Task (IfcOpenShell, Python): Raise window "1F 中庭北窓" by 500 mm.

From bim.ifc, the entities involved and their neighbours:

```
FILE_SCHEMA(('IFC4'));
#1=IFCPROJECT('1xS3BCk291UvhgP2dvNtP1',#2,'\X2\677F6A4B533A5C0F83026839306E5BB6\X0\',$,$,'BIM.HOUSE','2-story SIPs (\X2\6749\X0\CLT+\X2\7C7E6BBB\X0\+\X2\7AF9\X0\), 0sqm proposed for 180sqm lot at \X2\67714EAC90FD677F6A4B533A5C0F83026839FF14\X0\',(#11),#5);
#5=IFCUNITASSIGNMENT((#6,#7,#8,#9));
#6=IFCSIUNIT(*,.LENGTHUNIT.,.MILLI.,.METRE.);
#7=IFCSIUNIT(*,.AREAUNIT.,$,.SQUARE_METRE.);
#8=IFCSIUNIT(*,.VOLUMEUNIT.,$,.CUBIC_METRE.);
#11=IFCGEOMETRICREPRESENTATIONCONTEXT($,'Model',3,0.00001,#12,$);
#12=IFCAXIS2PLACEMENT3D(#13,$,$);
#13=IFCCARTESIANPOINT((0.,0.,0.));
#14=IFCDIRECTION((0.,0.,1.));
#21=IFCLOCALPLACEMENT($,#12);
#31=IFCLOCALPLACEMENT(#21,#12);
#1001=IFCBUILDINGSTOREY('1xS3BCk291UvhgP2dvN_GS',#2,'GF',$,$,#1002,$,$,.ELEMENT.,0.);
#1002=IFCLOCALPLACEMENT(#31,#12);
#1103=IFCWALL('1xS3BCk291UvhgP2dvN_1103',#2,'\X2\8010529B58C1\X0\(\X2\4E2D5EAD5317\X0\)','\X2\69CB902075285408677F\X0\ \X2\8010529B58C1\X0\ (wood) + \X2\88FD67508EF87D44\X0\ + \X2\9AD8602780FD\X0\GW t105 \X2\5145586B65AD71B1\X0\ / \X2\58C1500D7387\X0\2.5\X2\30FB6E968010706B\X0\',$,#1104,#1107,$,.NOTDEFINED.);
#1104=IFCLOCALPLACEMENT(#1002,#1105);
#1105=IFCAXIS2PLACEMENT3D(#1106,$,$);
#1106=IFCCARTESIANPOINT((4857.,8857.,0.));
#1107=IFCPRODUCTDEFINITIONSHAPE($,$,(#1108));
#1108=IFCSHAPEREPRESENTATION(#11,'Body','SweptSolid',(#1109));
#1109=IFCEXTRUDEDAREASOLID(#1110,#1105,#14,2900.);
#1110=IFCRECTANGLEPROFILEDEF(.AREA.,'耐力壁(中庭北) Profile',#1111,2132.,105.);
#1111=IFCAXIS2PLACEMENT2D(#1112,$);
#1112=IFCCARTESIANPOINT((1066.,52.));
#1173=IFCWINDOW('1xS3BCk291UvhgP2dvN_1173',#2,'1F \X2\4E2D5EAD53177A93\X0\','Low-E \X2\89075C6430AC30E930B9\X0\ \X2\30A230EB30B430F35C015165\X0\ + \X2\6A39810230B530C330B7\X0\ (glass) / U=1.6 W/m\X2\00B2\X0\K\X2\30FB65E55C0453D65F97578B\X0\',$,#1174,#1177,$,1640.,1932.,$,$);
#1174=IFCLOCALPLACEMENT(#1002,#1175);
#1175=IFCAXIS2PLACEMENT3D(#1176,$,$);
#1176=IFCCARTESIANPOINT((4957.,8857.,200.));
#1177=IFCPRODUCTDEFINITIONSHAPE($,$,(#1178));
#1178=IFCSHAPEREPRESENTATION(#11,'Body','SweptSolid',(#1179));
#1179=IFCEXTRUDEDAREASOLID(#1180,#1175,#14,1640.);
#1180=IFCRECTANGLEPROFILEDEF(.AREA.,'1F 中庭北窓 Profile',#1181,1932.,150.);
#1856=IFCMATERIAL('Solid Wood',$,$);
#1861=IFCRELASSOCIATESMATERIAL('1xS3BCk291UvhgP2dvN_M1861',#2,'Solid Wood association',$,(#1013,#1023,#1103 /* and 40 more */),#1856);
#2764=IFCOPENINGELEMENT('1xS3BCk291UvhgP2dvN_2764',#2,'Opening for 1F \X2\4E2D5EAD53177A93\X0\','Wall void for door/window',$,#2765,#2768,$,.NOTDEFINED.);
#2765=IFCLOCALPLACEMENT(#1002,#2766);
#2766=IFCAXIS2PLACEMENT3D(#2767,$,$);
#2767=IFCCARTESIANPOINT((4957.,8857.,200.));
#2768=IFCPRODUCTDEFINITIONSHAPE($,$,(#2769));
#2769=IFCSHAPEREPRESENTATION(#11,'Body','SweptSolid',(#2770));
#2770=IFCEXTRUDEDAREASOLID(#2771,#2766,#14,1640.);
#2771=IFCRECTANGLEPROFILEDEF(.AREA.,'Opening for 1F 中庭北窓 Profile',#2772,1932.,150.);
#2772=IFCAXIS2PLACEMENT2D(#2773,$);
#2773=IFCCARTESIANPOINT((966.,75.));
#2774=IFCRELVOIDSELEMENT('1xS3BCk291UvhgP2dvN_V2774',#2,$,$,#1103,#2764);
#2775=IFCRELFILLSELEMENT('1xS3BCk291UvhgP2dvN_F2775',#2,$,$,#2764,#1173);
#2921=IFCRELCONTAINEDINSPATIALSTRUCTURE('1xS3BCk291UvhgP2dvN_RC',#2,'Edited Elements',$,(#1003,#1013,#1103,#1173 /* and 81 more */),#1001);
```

```python
import numpy as np
import ifcopenshell
import ifcopenshell.api.geometry
import ifcopenshell.util.placement
import ifcopenshell.util.unit

model = ifcopenshell.open("bim.ifc")
unit_scale = ifcopenshell.util.unit.calculate_unit_scale(model)

window = model.by_guid("1xS3BCk291UvhgP2dvN_1173")
opening = window.FillsVoids[0].RelatingOpeningElement
dz = 0.5 / unit_scale

shift = np.array([0.0, 0.0, dz])
# The window is not placed relative to its opening, so move both.
for product in (opening, window):
    matrix = ifcopenshell.util.placement.get_local_placement(product.ObjectPlacement)
    matrix[:3, 3] += shift
    ifcopenshell.api.geometry.edit_object_placement(model, product=product, matrix=matrix, is_si=False)

print(f"moved by {dz * unit_scale:+.3f} m")

model.write("bim-out.ifc")
```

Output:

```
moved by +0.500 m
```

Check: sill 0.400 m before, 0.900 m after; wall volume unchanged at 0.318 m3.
